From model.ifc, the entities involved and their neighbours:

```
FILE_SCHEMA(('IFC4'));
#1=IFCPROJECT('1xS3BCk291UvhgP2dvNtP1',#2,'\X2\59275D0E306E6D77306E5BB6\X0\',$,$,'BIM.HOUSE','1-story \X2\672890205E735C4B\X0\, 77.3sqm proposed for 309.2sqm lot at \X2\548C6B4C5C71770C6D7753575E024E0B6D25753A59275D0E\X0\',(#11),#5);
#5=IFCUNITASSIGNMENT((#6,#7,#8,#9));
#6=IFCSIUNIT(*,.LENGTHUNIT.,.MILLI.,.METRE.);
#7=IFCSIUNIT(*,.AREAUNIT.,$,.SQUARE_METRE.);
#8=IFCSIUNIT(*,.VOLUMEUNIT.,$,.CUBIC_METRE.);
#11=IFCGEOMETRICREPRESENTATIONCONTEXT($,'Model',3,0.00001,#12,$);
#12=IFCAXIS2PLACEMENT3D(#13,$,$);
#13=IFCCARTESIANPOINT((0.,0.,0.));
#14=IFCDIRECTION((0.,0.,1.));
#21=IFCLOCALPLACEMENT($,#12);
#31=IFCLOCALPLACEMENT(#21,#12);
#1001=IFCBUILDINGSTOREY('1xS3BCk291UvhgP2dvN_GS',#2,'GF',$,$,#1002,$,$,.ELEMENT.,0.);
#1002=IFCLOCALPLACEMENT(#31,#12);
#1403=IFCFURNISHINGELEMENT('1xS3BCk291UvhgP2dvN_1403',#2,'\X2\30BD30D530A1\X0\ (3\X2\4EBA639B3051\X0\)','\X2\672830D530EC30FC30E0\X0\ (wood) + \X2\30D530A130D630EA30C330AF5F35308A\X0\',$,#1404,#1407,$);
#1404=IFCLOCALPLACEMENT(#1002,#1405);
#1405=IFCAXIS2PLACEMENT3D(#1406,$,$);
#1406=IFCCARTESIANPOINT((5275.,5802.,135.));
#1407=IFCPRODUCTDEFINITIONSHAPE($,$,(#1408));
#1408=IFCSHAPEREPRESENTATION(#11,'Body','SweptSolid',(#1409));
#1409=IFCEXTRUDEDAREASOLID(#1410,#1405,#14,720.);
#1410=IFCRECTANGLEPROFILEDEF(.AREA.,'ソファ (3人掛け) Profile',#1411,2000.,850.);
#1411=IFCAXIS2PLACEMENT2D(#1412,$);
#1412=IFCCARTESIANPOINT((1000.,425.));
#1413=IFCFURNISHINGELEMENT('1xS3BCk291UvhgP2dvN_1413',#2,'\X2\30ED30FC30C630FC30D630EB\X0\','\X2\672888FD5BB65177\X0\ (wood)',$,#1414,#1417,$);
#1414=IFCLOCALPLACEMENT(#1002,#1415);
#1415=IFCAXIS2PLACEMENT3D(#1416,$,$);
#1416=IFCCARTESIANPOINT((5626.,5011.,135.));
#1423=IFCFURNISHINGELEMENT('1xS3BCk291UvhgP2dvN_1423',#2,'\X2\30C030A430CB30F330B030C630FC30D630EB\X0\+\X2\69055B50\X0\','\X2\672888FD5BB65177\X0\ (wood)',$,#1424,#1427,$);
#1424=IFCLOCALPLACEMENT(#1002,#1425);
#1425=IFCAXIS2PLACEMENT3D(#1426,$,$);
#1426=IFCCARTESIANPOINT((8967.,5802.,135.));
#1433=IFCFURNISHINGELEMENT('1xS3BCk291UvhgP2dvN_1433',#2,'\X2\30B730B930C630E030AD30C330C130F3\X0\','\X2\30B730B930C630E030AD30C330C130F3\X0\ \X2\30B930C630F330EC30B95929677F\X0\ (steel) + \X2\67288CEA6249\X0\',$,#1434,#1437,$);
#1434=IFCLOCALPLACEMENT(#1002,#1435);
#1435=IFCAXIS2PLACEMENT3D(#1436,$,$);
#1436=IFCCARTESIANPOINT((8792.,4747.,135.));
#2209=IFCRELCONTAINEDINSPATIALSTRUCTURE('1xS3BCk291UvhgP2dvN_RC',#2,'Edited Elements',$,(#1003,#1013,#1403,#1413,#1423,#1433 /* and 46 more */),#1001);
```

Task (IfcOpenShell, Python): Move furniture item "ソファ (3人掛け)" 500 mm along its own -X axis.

```python
import ifcopenshell
import ifcopenshell.api.geometry
import ifcopenshell.util.placement

model = ifcopenshell.open("model.ifc")

item = model.by_id(1403)
matrix = ifcopenshell.util.placement.get_local_placement(item.ObjectPlacement)
matrix[:3, 3] -= matrix[:3, 0] * 500.0
ifcopenshell.api.geometry.edit_object_placement(model, product=item, matrix=matrix, is_si=False)

print(ifcopenshell.util.placement.get_local_placement(item.ObjectPlacement).round(3) + 0.0)

model.write("model-out.ifc")
```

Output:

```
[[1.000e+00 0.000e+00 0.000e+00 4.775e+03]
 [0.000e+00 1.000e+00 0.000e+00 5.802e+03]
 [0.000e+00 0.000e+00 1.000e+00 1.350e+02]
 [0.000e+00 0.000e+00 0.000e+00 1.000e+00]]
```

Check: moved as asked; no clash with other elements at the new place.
